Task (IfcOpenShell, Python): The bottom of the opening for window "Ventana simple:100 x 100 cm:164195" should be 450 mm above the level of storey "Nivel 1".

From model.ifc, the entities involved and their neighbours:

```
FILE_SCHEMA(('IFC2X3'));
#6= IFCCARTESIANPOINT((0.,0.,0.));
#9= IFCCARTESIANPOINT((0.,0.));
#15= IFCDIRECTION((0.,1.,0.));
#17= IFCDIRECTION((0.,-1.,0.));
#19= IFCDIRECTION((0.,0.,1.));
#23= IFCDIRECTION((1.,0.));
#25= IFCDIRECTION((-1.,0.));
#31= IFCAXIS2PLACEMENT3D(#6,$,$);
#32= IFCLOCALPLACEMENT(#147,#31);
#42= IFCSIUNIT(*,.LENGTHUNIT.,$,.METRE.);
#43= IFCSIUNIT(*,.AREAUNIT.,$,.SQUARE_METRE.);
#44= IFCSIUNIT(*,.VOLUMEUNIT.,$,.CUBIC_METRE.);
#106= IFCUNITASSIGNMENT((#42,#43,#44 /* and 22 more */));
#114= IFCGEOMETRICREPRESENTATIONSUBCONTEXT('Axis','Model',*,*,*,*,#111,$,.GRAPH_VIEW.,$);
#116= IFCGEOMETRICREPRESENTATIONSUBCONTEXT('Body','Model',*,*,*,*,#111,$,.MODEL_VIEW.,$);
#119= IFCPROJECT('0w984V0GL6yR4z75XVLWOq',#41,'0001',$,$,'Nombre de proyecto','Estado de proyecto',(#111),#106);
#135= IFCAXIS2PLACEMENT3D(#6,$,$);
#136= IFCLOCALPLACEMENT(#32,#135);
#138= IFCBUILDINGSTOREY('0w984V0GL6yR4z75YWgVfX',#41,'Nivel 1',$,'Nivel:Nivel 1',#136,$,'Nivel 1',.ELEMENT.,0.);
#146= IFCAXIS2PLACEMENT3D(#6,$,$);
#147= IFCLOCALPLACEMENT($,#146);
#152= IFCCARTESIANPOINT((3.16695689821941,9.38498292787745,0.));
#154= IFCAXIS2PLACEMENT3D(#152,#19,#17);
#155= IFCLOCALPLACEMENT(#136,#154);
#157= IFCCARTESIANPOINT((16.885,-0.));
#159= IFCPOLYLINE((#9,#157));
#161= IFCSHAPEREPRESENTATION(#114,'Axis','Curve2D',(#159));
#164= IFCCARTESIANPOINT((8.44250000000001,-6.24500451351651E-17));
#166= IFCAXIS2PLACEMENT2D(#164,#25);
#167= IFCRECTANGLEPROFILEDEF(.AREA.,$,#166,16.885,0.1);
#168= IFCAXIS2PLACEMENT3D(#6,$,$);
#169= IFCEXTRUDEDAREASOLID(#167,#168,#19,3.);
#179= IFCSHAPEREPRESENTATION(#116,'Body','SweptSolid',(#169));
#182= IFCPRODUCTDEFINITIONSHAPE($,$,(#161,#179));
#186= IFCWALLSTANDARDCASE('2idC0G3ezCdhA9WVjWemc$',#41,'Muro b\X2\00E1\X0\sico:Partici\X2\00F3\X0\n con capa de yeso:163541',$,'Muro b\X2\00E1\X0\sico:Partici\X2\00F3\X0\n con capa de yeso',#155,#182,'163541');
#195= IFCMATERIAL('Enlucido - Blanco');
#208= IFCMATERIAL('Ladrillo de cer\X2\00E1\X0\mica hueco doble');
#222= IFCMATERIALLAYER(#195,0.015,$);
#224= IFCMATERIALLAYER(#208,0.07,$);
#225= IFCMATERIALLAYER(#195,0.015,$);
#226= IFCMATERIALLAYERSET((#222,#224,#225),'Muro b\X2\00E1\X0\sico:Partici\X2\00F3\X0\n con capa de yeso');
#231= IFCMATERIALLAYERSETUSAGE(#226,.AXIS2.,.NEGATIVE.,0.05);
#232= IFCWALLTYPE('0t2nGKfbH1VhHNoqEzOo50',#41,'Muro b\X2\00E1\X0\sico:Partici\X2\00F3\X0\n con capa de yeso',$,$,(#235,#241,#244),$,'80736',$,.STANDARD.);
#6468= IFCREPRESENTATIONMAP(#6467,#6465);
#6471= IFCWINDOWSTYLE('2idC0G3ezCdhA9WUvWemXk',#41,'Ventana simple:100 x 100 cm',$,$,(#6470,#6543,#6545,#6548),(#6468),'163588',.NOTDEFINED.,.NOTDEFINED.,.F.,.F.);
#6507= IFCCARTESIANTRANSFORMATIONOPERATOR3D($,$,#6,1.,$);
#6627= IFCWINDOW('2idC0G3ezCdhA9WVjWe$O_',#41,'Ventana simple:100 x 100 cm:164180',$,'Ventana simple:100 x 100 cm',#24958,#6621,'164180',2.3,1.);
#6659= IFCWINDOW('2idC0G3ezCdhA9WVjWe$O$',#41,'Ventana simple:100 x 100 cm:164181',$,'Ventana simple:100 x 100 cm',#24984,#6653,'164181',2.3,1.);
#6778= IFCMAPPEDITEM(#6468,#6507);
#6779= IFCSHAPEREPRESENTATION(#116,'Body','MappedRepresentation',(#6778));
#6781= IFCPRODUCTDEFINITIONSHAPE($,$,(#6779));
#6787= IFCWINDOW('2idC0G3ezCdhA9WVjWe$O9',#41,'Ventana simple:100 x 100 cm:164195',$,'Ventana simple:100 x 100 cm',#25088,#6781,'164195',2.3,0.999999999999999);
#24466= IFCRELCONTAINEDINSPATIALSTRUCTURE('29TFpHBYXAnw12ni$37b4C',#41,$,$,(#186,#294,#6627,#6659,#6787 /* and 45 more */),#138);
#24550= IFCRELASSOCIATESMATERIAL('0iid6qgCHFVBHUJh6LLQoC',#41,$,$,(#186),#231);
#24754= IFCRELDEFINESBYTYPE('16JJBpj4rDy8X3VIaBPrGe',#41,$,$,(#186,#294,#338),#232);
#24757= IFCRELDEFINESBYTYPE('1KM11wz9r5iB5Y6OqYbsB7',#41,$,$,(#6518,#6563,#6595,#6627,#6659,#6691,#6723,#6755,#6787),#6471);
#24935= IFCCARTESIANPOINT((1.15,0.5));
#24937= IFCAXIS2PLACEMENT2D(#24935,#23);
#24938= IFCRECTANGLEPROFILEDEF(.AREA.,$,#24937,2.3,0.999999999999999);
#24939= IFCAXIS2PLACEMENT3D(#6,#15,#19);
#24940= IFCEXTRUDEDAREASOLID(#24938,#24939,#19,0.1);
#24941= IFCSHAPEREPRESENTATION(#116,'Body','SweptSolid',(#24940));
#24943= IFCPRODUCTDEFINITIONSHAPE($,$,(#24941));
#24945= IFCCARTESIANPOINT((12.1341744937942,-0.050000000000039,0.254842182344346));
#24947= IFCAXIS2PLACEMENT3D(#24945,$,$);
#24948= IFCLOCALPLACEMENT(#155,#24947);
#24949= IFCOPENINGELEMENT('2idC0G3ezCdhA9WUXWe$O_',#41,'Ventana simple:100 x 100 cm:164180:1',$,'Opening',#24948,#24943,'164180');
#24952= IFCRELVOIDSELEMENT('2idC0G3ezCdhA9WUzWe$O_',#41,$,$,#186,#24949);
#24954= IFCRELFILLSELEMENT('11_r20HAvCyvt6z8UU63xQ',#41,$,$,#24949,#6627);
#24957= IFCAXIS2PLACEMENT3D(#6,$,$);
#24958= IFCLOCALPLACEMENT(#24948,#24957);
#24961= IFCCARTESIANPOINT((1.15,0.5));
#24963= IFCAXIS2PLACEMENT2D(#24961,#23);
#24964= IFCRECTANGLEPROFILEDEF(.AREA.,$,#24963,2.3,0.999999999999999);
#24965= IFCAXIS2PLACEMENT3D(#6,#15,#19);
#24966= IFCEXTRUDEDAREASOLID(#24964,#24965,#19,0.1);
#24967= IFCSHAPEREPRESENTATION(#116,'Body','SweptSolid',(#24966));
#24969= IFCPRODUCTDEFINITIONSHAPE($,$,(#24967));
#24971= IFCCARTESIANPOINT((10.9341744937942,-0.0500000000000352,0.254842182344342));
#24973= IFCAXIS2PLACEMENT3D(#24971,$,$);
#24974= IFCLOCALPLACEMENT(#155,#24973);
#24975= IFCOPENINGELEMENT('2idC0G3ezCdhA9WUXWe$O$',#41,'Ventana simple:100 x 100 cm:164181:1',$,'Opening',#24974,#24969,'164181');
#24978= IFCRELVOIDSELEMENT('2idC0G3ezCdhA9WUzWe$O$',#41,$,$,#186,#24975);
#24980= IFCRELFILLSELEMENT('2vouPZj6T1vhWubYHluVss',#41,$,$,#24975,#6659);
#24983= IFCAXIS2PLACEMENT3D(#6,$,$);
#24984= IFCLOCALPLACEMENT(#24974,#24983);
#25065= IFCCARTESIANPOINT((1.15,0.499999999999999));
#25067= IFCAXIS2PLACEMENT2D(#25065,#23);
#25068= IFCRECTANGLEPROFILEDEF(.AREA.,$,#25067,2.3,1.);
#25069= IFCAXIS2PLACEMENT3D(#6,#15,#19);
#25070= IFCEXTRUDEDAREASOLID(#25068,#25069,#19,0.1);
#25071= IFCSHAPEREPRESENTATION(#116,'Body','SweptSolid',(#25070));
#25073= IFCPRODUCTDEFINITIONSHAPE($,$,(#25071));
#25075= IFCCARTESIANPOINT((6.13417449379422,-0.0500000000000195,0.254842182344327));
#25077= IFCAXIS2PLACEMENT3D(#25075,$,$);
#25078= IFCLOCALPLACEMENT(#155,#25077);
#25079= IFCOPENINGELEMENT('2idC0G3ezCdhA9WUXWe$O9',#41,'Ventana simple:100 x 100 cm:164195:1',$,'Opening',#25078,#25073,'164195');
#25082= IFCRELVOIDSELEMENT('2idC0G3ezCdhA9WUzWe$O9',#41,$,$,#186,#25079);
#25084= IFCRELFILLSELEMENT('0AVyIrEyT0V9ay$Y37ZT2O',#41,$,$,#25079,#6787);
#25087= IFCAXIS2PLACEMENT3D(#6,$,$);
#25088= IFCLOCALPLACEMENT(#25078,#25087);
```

```python
import numpy as np
import ifcopenshell
import ifcopenshell.api.geometry
import ifcopenshell.geom
import ifcopenshell.util.element
import ifcopenshell.util.placement
import ifcopenshell.util.shape
import ifcopenshell.util.unit

model = ifcopenshell.open("model.ifc")
unit_scale = ifcopenshell.util.unit.calculate_unit_scale(model)

window = model.by_guid("2idC0G3ezCdhA9WVjWe$O9")
opening = window.FillsVoids[0].RelatingOpeningElement
storey = ifcopenshell.util.element.get_container(window, ifc_class="IfcBuildingStorey")
level = ifcopenshell.util.placement.get_local_placement(storey.ObjectPlacement)[2, 3]

# The opening's origin need not be at the sill, so measure its lowest point.
shape = ifcopenshell.geom.create_shape(ifcopenshell.geom.settings(), opening)
bottom = ifcopenshell.util.shape.get_shape_bottom_elevation(shape, shape.geometry) / unit_scale
dz = level + 0.45 - bottom

shift = np.array([0.0, 0.0, dz])
# The window is placed relative to its opening, so it follows when the opening moves.
matrix = ifcopenshell.util.placement.get_local_placement(opening.ObjectPlacement)
matrix[:3, 3] += shift
ifcopenshell.api.geometry.edit_object_placement(
    model, product=opening, matrix=matrix, is_si=False, should_transform_children=True
)

print(f"moved by {dz * unit_scale:+.3f} m")

model.write("model_rev.ifc")
```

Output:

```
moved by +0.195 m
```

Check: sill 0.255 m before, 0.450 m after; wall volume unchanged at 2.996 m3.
